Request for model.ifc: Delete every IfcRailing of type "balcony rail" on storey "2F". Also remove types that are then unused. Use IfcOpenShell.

First a look at what the model holds.

```python
import ifcopenshell
import ifcopenshell.util.element

model = ifcopenshell.open("model.ifc")
print(model.schema)
storey = next(s for s in model.by_type("IfcBuildingStorey") if s.Name == "2F")
railings = [e for e in ifcopenshell.util.element.get_decomposition(storey) if e.is_a("IfcRailing")]
seen = {}
for e in railings:
    element_type = ifcopenshell.util.element.get_type(e)
    name = element_type.Name if element_type not in (None, e) else None
    seen[name] = seen.get(name, 0) + 1
for name, count in sorted(seen.items(), key=str):
    print(count, "x", name)
```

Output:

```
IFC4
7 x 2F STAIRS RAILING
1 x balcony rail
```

```python
import ifcopenshell
import ifcopenshell.api.root
import ifcopenshell.util.element

model = ifcopenshell.open("model.ifc")

storey = next(s for s in model.by_type("IfcBuildingStorey") if s.Name == "2F")
railings = [e for e in ifcopenshell.util.element.get_decomposition(storey) if e.is_a("IfcRailing")]
targets = [e for e in railings if (t := ifcopenshell.util.element.get_type(e)) not in (None, e) and t.Name == "balcony rail"]
types = {ifcopenshell.util.element.get_type(e) for e in targets} - {None, *targets}

for e in targets:
    ifcopenshell.api.root.remove_product(model, product=e)
print(len(targets), "removed")

unused = [t for t in types if not ifcopenshell.util.element.get_types(t)]
for t in unused:
    ifcopenshell.api.root.remove_product(model, product=t)
print(len(unused), "unused types removed")

model.write("model_edited.ifc")
```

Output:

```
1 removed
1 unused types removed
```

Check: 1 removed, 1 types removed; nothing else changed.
